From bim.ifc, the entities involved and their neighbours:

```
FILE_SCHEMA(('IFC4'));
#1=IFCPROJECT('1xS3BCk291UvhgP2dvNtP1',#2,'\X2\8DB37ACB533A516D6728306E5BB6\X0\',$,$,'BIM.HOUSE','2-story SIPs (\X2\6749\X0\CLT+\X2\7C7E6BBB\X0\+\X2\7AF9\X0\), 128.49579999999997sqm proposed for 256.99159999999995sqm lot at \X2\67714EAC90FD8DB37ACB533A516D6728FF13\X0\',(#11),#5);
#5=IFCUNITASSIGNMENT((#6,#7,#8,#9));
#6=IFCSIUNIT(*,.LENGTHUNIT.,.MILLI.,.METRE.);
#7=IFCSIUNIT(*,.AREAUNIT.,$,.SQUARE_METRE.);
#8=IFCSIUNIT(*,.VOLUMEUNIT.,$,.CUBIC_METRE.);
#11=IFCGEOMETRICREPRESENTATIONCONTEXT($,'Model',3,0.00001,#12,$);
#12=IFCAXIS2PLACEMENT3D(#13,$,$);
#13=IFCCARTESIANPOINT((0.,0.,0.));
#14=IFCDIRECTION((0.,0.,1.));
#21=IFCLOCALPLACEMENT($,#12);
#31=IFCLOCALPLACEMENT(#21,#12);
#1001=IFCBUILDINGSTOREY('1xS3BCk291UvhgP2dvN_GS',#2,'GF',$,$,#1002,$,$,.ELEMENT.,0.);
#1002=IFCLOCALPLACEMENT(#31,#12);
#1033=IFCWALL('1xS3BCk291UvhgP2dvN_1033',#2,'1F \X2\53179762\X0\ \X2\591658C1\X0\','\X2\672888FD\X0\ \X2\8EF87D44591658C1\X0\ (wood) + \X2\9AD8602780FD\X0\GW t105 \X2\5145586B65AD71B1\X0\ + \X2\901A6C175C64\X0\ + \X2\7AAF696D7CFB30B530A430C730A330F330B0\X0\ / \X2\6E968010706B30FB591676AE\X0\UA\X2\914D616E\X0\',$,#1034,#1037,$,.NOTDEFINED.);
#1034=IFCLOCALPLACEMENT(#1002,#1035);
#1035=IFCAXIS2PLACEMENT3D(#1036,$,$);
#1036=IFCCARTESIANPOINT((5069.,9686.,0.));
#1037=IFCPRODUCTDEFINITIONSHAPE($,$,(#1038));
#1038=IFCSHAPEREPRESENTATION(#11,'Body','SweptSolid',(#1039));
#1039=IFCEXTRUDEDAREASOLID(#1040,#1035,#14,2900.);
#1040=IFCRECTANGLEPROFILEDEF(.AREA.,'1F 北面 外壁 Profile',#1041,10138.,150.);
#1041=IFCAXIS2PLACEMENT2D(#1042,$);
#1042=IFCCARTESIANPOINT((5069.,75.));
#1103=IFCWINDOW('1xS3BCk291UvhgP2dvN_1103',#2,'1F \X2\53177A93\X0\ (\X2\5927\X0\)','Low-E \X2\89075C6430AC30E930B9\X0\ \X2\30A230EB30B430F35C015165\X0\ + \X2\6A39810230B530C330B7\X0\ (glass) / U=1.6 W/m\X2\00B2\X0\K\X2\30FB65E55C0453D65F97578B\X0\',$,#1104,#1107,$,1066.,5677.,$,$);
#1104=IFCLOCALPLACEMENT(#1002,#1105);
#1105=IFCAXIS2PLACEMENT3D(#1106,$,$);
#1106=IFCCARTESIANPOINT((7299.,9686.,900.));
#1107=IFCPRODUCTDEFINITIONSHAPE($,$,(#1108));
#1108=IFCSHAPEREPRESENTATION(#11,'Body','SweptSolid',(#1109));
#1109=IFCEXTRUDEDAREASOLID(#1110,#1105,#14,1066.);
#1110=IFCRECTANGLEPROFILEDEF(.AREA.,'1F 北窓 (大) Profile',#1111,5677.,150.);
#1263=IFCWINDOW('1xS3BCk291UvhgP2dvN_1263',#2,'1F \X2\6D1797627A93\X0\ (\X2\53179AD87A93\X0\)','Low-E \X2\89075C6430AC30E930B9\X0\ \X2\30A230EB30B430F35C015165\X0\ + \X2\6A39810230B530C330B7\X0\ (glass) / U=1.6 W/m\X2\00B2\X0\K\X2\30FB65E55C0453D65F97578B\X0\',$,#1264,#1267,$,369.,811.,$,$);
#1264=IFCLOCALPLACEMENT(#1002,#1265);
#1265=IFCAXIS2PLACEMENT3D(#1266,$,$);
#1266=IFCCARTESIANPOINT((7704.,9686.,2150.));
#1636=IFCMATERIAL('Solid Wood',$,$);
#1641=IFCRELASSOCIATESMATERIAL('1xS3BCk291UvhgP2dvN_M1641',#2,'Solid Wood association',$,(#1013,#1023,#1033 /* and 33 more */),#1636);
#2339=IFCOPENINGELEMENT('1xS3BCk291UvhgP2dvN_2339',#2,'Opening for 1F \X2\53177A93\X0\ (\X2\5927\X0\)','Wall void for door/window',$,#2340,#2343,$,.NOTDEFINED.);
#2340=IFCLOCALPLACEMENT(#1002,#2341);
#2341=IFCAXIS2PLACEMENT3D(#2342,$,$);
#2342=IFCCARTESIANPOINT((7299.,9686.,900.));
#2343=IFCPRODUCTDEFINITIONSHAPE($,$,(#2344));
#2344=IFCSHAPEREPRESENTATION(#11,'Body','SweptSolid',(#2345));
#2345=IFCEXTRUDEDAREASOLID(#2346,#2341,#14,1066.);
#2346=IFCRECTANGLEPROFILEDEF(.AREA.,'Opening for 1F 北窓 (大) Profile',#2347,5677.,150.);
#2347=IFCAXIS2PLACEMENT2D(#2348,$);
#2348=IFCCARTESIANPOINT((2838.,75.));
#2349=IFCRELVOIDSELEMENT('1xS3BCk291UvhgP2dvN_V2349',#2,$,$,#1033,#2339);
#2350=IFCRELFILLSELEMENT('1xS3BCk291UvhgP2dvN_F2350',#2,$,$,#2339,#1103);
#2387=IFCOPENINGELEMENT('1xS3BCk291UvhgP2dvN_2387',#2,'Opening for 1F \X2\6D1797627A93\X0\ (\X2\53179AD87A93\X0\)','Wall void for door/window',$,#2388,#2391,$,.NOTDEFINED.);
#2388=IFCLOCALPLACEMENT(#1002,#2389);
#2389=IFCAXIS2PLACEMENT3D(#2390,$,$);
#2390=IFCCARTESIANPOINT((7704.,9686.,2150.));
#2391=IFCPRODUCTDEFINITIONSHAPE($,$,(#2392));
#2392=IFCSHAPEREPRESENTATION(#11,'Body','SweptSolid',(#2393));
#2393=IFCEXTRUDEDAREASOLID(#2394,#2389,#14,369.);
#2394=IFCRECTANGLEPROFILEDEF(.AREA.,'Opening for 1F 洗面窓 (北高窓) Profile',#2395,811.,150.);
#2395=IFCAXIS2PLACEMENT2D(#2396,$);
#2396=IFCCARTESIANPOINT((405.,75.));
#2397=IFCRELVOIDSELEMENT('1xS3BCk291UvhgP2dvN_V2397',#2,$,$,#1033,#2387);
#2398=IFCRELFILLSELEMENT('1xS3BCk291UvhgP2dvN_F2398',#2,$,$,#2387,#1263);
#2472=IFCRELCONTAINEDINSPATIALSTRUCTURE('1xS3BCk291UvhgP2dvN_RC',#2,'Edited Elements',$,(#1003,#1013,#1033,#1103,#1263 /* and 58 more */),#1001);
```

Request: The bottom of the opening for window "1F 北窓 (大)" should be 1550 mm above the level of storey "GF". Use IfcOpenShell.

```python
import numpy as np
import ifcopenshell
import ifcopenshell.api.geometry
import ifcopenshell.geom
import ifcopenshell.util.element
import ifcopenshell.util.placement
import ifcopenshell.util.shape
import ifcopenshell.util.unit

model = ifcopenshell.open("bim.ifc")
unit_scale = ifcopenshell.util.unit.calculate_unit_scale(model)

window = model.by_guid("1xS3BCk291UvhgP2dvN_1103")
opening = window.FillsVoids[0].RelatingOpeningElement
storey = ifcopenshell.util.element.get_container(window, ifc_class="IfcBuildingStorey")
level = ifcopenshell.util.placement.get_local_placement(storey.ObjectPlacement)[2, 3]

# The opening's origin need not be at the sill, so measure its lowest point.
shape = ifcopenshell.geom.create_shape(ifcopenshell.geom.settings(), opening)
bottom = ifcopenshell.util.shape.get_shape_bottom_elevation(shape, shape.geometry) / unit_scale
dz = level + 1.55 / unit_scale - bottom

shift = np.array([0.0, 0.0, dz])
# The window is not placed relative to its opening, so move both.
for product in (opening, window):
    matrix = ifcopenshell.util.placement.get_local_placement(product.ObjectPlacement)
    matrix[:3, 3] += shift
    ifcopenshell.api.geometry.edit_object_placement(model, product=product, matrix=matrix, is_si=False)

print(f"moved by {dz * unit_scale:+.3f} m")

model.write("bim_edited.ifc")
```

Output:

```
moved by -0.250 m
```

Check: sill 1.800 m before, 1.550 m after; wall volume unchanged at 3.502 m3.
